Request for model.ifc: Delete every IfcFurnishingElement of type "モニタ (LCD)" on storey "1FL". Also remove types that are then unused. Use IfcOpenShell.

First a look at what the model holds.

```python
import ifcopenshell
import ifcopenshell.util.element

model = ifcopenshell.open("model.ifc")
print(model.schema)
storey = next(s for s in model.by_type("IfcBuildingStorey") if s.Name == "1FL")
furniture = [e for e in ifcopenshell.util.element.get_decomposition(storey) if e.is_a("IfcFurnishingElement")]
seen = {}
for e in furniture:
    element_type = ifcopenshell.util.element.get_type(e)
    name = element_type.Name if element_type not in (None, e) else None
    seen[name] = seen.get(name, 0) + 1
for name, count in sorted(seen.items(), key=str):
    print(count, "x", name)
```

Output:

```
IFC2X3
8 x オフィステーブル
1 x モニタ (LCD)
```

```python
import ifcopenshell
import ifcopenshell.api.root
import ifcopenshell.util.element

model = ifcopenshell.open("model.ifc")

storey = next(s for s in model.by_type("IfcBuildingStorey") if s.Name == "1FL")
furniture = [e for e in ifcopenshell.util.element.get_decomposition(storey) if e.is_a("IfcFurnishingElement")]
targets = [e for e in furniture if (t := ifcopenshell.util.element.get_type(e)) not in (None, e) and t.Name == "モニタ (LCD)"]
types = {ifcopenshell.util.element.get_type(e) for e in targets} - {None, *targets}

for e in targets:
    ifcopenshell.api.root.remove_product(model, product=e)
print(len(targets), "removed")

unused = [t for t in types if not ifcopenshell.util.element.get_types(t)]
for t in unused:
    ifcopenshell.api.root.remove_product(model, product=t)
print(len(unused), "unused types removed")

model.write("model_updated.ifc")
```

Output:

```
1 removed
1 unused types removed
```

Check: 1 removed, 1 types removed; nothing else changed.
